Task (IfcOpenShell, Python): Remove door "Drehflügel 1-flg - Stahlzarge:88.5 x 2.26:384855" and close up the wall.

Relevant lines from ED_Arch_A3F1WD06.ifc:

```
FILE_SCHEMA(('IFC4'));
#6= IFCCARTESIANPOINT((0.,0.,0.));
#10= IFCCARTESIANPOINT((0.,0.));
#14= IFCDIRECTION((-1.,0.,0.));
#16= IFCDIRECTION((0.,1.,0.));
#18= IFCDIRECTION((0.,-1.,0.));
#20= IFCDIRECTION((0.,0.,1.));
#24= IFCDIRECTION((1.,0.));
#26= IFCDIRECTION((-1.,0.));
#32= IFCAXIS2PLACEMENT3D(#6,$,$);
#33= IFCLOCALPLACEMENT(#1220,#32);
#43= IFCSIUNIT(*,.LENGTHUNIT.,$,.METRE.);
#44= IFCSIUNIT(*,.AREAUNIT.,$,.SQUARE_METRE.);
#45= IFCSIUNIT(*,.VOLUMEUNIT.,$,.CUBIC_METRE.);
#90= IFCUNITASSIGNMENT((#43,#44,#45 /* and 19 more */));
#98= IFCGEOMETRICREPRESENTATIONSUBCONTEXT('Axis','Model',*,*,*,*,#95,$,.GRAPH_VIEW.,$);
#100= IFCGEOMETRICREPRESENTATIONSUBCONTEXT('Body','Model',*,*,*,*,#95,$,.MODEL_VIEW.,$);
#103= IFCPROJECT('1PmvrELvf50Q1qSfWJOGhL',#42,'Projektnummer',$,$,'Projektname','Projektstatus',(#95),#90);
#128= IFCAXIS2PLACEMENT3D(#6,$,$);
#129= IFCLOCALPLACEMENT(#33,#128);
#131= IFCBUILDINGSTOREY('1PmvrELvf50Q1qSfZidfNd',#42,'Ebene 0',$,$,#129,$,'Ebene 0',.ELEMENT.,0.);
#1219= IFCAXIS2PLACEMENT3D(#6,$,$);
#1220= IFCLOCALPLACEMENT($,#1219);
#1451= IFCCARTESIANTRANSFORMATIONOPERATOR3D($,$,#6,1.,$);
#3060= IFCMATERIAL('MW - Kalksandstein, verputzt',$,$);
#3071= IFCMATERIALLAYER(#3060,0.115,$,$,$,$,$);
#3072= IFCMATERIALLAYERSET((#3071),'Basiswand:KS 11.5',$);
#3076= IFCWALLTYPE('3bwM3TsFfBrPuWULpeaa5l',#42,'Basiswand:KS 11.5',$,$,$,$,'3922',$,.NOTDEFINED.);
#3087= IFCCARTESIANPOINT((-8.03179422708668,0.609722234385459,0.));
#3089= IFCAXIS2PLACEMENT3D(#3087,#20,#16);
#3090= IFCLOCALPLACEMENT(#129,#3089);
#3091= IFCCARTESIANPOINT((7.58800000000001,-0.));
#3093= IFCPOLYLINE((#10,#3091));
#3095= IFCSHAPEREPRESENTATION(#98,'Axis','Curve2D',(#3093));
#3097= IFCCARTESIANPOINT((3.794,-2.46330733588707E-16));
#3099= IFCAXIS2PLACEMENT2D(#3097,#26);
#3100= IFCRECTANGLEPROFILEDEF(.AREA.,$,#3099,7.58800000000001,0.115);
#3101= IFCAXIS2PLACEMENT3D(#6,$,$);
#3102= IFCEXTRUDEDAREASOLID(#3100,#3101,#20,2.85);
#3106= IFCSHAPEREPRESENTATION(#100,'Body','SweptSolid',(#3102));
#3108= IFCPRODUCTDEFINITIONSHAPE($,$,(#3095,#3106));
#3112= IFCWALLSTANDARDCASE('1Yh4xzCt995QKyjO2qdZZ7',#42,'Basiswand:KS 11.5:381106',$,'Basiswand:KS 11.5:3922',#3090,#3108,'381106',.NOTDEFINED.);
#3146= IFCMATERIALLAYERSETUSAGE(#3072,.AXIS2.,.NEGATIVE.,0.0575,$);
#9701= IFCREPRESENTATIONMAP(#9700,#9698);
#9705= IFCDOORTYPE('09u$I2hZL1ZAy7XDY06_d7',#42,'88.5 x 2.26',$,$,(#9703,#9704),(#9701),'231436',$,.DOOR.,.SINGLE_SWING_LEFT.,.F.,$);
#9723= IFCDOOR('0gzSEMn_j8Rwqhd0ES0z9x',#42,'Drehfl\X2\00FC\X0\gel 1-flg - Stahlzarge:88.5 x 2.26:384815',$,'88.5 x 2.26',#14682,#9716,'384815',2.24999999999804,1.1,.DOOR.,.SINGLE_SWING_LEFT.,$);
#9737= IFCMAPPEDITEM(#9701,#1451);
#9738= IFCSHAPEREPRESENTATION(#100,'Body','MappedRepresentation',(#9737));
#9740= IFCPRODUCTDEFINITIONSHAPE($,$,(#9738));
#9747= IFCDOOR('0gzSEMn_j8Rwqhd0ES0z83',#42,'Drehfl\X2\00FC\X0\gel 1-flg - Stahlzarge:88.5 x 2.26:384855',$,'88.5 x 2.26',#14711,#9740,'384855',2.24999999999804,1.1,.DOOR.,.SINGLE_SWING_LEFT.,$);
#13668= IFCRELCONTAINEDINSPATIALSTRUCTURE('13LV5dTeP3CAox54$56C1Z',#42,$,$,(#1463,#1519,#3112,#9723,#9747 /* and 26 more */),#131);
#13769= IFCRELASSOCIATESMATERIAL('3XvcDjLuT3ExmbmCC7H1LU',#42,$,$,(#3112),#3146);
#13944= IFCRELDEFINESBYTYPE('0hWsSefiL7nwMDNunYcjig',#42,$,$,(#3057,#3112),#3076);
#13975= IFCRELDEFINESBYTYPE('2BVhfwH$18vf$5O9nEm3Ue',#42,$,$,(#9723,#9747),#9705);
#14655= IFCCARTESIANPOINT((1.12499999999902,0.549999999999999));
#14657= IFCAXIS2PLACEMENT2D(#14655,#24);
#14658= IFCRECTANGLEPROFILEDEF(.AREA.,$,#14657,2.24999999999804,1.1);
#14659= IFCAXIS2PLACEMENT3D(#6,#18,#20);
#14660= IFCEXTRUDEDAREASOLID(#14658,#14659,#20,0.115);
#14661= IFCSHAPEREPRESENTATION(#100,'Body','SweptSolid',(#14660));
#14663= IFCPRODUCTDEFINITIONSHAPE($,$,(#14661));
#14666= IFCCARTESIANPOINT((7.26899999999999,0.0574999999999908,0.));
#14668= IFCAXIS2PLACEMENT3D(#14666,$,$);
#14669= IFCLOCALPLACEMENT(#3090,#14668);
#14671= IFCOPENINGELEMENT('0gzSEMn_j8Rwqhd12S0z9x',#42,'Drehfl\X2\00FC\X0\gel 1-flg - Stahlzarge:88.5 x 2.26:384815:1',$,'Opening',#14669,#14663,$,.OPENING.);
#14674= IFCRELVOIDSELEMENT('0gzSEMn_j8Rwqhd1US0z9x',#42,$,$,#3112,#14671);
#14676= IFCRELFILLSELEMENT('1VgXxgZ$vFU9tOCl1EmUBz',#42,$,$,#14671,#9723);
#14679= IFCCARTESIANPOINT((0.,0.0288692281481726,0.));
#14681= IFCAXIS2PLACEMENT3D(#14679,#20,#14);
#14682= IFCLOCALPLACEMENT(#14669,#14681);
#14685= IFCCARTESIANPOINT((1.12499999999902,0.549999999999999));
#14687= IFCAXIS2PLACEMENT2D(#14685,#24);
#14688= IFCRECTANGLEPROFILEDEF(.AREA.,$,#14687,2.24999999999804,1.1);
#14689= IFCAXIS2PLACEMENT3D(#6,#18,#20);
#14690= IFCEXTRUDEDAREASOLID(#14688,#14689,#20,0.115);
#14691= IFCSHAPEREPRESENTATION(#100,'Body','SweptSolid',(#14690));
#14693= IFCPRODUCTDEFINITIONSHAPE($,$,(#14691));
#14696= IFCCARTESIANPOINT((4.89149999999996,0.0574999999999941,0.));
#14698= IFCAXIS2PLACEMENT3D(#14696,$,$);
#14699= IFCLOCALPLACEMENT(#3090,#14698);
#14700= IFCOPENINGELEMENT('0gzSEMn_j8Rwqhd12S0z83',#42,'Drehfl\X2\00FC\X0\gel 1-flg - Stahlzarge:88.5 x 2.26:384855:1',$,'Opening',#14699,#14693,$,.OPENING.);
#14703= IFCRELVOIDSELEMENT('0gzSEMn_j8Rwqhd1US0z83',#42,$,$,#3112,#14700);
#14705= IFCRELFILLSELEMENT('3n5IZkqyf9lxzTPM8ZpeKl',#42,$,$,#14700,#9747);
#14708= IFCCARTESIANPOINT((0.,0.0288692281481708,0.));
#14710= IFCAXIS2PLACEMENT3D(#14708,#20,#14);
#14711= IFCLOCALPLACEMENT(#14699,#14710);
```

```python
import ifcopenshell
import ifcopenshell.api.feature
import ifcopenshell.api.root
import ifcopenshell.geom
import ifcopenshell.util.shape

model = ifcopenshell.open("ED_Arch_A3F1WD06.ifc")
settings = ifcopenshell.geom.settings()


def volume(element):
    """Net volume in cubic metres, openings subtracted."""
    shape = ifcopenshell.geom.create_shape(settings, element)
    return ifcopenshell.util.shape.get_volume(shape.geometry)


door = model.by_guid("0gzSEMn_j8Rwqhd0ES0z83")
opening = door.FillsVoids[0].RelatingOpeningElement
wall = opening.VoidsElements[0].RelatingBuildingElement
before = volume(wall)

ifcopenshell.api.root.remove_product(model, product=door)
ifcopenshell.api.feature.remove_feature(model, feature=opening)

after = volume(wall)

print(f"wall volume {before:.3f} -> {after:.3f} m3")

model.write("ED_Arch_A3F1WD06_rev.ifc")
```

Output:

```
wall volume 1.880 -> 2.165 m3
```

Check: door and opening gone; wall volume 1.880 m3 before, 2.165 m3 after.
